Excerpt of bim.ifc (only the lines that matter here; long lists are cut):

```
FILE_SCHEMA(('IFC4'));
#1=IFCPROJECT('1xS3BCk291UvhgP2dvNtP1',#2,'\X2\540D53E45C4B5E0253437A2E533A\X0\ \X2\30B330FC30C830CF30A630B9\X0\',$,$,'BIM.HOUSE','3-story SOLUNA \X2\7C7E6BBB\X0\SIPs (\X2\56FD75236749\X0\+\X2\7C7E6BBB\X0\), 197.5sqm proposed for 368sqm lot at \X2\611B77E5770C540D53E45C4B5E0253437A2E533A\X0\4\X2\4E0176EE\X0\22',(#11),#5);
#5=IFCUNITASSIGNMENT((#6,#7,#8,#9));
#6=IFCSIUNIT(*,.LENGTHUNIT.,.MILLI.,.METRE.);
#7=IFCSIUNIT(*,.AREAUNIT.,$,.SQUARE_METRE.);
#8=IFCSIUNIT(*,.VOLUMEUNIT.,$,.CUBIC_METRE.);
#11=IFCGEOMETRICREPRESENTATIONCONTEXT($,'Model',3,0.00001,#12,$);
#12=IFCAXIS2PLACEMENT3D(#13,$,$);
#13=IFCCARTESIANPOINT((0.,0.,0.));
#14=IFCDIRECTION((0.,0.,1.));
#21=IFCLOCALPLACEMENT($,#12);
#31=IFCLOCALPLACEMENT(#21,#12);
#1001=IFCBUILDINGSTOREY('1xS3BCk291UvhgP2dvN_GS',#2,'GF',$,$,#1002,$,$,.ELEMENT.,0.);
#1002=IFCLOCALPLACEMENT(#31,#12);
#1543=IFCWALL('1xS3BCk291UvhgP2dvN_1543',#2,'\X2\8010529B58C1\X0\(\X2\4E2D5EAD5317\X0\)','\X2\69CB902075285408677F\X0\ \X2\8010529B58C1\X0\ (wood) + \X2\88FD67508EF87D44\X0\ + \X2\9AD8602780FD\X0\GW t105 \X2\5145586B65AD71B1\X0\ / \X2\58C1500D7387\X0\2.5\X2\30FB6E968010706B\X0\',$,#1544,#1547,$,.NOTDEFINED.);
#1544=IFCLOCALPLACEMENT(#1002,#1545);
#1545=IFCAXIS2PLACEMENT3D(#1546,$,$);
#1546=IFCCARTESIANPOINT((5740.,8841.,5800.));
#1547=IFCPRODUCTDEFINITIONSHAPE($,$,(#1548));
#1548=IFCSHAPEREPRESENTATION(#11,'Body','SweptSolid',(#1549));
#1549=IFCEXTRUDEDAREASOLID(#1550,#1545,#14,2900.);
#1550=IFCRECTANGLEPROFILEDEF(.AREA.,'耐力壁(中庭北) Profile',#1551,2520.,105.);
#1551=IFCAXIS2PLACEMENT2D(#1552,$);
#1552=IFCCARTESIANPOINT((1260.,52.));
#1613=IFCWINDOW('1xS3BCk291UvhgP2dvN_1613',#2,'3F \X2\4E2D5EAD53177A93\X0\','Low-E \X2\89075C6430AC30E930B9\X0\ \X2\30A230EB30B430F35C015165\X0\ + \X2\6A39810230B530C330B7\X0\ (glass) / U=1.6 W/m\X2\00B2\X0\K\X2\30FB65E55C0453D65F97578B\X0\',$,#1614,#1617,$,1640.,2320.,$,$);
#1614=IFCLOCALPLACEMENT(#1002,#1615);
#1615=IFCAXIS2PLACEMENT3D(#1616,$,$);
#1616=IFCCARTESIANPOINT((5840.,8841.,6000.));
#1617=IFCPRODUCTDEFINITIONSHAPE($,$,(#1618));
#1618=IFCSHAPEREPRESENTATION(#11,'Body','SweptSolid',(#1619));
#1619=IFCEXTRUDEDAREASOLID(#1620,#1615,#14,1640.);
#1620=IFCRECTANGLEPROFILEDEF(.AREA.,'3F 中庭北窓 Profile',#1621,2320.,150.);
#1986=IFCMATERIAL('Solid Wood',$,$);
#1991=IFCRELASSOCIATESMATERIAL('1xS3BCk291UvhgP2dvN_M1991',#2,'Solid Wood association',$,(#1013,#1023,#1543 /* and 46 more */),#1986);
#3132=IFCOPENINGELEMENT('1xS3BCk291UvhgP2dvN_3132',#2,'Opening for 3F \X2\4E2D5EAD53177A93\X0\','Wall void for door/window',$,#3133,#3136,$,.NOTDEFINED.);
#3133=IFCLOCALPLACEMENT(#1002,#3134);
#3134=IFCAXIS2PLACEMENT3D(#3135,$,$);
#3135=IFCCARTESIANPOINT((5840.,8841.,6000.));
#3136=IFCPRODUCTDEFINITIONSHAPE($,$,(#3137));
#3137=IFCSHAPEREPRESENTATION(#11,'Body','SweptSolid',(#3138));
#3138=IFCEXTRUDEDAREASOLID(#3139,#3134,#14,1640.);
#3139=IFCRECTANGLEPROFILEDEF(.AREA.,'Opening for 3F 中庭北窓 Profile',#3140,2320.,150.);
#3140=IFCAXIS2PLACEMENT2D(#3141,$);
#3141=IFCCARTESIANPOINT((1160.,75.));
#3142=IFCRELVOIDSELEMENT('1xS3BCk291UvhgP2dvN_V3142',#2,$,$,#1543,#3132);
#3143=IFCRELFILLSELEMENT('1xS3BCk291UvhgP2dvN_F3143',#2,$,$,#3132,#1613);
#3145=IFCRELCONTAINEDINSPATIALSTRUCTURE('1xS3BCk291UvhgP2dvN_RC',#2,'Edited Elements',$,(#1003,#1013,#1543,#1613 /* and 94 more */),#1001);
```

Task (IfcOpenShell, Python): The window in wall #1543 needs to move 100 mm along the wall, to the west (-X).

```python
import ifcopenshell
import ifcopenshell.api.geometry
import ifcopenshell.util.placement
import ifcopenshell.util.unit

model = ifcopenshell.open("bim.ifc")
unit_scale = ifcopenshell.util.unit.calculate_unit_scale(model)

window = model.by_guid("1xS3BCk291UvhgP2dvN_1613")
opening = window.FillsVoids[0].RelatingOpeningElement
wall = opening.VoidsElements[0].RelatingBuildingElement

wall_matrix = ifcopenshell.util.placement.get_local_placement(wall.ObjectPlacement)
shift = wall_matrix[:3, 0] * -0.1 / unit_scale
before = ifcopenshell.util.placement.get_local_placement(window.ObjectPlacement)[:3, 3].copy()

# The window is not placed relative to its opening, so move both.
for product in (opening, window):
    matrix = ifcopenshell.util.placement.get_local_placement(product.ObjectPlacement)
    matrix[:3, 3] += shift
    ifcopenshell.api.geometry.edit_object_placement(model, product=product, matrix=matrix, is_si=False)

after = ifcopenshell.util.placement.get_local_placement(window.ObjectPlacement)[:3, 3]
print("window moved by", (after - before).round(3) + 0.0)

model.write("bim-out.ifc")
```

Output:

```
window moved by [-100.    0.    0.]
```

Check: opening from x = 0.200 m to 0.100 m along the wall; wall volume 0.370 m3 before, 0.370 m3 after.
